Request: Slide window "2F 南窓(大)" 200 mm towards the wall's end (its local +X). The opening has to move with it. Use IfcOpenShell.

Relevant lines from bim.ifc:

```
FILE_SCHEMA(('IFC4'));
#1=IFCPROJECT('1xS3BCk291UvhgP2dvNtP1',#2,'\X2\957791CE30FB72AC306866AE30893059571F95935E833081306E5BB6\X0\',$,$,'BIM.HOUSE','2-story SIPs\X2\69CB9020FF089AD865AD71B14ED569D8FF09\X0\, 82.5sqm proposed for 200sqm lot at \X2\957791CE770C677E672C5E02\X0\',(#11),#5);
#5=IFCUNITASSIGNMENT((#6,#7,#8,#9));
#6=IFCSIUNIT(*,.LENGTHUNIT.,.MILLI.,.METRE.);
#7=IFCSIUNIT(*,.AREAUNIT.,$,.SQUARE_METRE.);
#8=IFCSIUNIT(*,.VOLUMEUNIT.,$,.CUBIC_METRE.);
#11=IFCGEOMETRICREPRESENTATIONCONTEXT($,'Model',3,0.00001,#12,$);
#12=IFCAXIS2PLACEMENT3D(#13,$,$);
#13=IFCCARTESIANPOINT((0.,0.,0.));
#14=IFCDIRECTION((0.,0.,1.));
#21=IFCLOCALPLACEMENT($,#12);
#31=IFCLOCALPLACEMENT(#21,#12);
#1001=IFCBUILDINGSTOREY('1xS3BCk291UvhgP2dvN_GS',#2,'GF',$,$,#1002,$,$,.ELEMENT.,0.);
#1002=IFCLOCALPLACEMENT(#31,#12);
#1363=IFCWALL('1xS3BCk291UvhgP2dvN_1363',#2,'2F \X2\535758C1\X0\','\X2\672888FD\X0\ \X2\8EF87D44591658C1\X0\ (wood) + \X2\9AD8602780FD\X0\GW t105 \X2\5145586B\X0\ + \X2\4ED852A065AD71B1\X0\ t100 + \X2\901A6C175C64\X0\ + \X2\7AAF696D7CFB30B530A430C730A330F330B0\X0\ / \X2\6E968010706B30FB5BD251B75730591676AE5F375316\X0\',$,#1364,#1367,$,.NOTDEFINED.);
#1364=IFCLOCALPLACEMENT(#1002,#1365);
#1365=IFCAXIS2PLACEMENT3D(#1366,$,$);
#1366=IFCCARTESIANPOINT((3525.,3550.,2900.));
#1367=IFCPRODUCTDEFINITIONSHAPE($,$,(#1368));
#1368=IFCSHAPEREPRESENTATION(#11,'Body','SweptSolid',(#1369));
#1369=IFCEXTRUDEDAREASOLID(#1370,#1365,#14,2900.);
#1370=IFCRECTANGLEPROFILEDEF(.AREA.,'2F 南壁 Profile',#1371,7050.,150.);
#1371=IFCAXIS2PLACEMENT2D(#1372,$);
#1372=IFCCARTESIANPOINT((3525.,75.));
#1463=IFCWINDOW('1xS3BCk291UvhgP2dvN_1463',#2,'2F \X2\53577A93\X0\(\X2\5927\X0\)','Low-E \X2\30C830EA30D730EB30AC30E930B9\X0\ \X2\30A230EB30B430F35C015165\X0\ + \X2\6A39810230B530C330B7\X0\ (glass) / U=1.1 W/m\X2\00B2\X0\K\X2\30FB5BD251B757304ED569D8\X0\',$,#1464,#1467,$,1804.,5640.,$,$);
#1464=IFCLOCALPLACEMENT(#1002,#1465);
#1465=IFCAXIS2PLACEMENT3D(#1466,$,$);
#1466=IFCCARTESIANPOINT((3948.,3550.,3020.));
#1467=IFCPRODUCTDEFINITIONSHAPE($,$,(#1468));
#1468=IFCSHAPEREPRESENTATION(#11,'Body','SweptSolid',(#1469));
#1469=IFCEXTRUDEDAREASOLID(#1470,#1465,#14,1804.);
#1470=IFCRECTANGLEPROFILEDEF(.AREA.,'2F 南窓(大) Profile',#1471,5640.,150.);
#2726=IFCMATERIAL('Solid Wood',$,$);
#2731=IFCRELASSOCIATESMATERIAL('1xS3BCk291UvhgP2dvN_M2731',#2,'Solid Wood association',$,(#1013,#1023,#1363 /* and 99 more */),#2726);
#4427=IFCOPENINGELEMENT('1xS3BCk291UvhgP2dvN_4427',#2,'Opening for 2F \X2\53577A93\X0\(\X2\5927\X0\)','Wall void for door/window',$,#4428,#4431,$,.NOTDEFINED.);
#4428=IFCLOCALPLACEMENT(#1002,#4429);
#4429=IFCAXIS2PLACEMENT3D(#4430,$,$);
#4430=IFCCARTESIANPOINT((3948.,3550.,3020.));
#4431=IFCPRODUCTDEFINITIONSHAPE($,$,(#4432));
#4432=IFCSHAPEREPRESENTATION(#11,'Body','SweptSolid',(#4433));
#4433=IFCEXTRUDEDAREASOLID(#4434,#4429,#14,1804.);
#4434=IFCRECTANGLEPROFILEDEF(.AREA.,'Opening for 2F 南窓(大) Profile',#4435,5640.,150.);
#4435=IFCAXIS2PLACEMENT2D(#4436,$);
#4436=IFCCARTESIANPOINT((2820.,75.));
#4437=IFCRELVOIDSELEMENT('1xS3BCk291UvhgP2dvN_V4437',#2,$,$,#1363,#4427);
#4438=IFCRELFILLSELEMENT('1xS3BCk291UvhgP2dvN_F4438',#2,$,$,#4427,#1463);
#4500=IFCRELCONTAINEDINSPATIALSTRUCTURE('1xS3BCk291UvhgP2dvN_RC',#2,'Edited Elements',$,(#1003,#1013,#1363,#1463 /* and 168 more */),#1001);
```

```python
import ifcopenshell
import ifcopenshell.api.geometry
import ifcopenshell.util.placement
import ifcopenshell.util.unit

model = ifcopenshell.open("bim.ifc")
unit_scale = ifcopenshell.util.unit.calculate_unit_scale(model)

window = model.by_guid("1xS3BCk291UvhgP2dvN_1463")
opening = window.FillsVoids[0].RelatingOpeningElement
wall = opening.VoidsElements[0].RelatingBuildingElement

wall_matrix = ifcopenshell.util.placement.get_local_placement(wall.ObjectPlacement)
shift = wall_matrix[:3, 0] * 0.2 / unit_scale
before = ifcopenshell.util.placement.get_local_placement(window.ObjectPlacement)[:3, 3].copy()

# The window is not placed relative to its opening, so move both.
for product in (opening, window):
    matrix = ifcopenshell.util.placement.get_local_placement(product.ObjectPlacement)
    matrix[:3, 3] += shift
    ifcopenshell.api.geometry.edit_object_placement(model, product=product, matrix=matrix, is_si=False)

after = ifcopenshell.util.placement.get_local_placement(window.ObjectPlacement)[:3, 3]
print("window moved by", (after - before).round(3) + 0.0)

model.write("bim_v2.ifc")
```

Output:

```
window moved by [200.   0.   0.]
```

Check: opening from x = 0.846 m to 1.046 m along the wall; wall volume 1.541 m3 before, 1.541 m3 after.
